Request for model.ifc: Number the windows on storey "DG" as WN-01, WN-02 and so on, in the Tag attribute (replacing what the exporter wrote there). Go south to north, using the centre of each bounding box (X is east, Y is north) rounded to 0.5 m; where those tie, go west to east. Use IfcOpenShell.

First a look at what the model holds.

```python
import ifcopenshell
import ifcopenshell.util.element
import ifcopenshell.util.placement

model = ifcopenshell.open("model.ifc")
print(model.schema)
storey = next(s for s in model.by_type("IfcBuildingStorey") if s.Name == "DG")
windows = [e for e in ifcopenshell.util.element.get_decomposition(storey) if e.is_a("IfcWindow")]
for e in sorted(windows, key=lambda e: e.id()):
    origin = ifcopenshell.util.placement.get_local_placement(e.ObjectPlacement)[:3, 3]
    print(e.id(), e.Tag, e.Name, origin.round(2) + 0.0, sep=" | ")
```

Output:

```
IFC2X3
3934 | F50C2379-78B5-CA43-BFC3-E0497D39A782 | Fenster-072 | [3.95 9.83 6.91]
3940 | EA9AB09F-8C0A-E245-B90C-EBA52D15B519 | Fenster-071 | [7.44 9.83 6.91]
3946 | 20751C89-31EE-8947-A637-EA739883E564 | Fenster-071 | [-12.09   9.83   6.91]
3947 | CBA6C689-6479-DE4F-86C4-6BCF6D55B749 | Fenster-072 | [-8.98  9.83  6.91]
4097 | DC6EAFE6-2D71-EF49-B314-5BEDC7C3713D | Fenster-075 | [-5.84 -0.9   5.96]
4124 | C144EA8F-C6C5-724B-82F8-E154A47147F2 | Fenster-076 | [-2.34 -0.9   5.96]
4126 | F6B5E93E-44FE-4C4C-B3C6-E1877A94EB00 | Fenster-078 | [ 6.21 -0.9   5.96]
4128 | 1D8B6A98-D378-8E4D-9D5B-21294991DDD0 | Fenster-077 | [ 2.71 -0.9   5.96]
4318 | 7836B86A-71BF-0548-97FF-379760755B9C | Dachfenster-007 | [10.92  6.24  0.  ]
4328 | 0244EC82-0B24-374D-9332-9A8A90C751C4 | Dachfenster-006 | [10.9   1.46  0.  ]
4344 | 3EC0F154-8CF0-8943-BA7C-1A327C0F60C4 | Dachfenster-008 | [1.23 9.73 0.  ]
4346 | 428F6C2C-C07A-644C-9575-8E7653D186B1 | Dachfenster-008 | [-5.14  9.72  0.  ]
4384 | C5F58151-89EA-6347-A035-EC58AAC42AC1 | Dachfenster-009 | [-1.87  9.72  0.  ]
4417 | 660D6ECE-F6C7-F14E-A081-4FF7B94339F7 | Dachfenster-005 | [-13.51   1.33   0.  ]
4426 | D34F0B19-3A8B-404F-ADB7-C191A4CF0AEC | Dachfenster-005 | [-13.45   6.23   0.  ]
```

```python
import ifcopenshell
import ifcopenshell.geom
import ifcopenshell.util.element
import ifcopenshell.util.shape

model = ifcopenshell.open("model.ifc")
settings = ifcopenshell.geom.settings()
settings.set("use-world-coords", True)


def centre(element):
    shape = ifcopenshell.geom.create_shape(settings, element)
    return ifcopenshell.util.shape.get_bbox_centroid(shape.geometry)


storey = next(s for s in model.by_type("IfcBuildingStorey") if s.Name == "DG")
windows = [e for e in ifcopenshell.util.element.get_decomposition(storey) if e.is_a("IfcWindow")]

# Insertion points can sit at a corner or the storey origin, so sort by the geometry (in metres).
centres = {e: centre(e) for e in windows}
windows.sort(key=lambda e: (round(centres[e][1] / 0.5), centres[e][0]))

for i, e in enumerate(windows, start=1):
    number = f"WN-{i:02d}"
    e.Tag = number
    print(e.id(), number)

model.write("model_edited.ifc")
```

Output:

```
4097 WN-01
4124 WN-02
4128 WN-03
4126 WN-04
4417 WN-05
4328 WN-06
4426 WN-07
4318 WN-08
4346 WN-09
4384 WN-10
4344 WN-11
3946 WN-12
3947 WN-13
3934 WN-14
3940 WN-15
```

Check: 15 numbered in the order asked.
